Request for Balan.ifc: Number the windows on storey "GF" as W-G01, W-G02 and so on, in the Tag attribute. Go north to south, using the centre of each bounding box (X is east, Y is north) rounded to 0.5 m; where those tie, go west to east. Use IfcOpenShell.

First a look at what the model holds.

```python
import ifcopenshell
import ifcopenshell.util.element
import ifcopenshell.util.placement

model = ifcopenshell.open("Balan.ifc")
print(model.schema)
storey = next(s for s in model.by_type("IfcBuildingStorey") if s.Name == "GF")
windows = [e for e in ifcopenshell.util.element.get_decomposition(storey) if e.is_a("IfcWindow")]
for e in sorted(windows, key=lambda e: e.id()):
    origin = ifcopenshell.util.placement.get_local_placement(e.ObjectPlacement)[:3, 3]
    print(e.id(), e.Tag, e.Name, origin.round(2) + 0.0, sep=" | ")
```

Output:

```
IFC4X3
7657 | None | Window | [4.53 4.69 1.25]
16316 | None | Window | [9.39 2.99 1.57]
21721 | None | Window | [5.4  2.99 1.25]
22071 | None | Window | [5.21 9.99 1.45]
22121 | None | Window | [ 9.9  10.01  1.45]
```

```python
import ifcopenshell
import ifcopenshell.geom
import ifcopenshell.util.element
import ifcopenshell.util.shape

model = ifcopenshell.open("Balan.ifc")
settings = ifcopenshell.geom.settings()
settings.set("use-world-coords", True)


def centre(element):
    shape = ifcopenshell.geom.create_shape(settings, element)
    return ifcopenshell.util.shape.get_bbox_centroid(shape.geometry)


storey = next(s for s in model.by_type("IfcBuildingStorey") if s.Name == "GF")
windows = [e for e in ifcopenshell.util.element.get_decomposition(storey) if e.is_a("IfcWindow")]

# Insertion points can sit at a corner or the storey origin, so sort by the geometry (in metres).
centres = {e: centre(e) for e in windows}
windows.sort(key=lambda e: (-round(centres[e][1] / 0.5), centres[e][0]))

for i, e in enumerate(windows, start=1):
    number = f"W-G{i:02d}"
    e.Tag = number
    print(e.id(), number)

model.write("Balan_rev.ifc")
```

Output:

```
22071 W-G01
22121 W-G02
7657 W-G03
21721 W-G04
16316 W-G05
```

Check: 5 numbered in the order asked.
